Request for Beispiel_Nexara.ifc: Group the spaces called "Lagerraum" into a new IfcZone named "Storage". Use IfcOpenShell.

First a look at what the model holds.

```python
import ifcopenshell

model = ifcopenshell.open("Beispiel_Nexara.ifc")
print(model.schema)
seen = {}
for space in model.by_type("IfcSpace"):
    seen[space.LongName] = seen.get(space.LongName, 0) + 1
for name, count in sorted(seen.items(), key=str):
    print(count, "x", name)
print("zones:", [z.Name for z in model.by_type("IfcZone")][:20])
```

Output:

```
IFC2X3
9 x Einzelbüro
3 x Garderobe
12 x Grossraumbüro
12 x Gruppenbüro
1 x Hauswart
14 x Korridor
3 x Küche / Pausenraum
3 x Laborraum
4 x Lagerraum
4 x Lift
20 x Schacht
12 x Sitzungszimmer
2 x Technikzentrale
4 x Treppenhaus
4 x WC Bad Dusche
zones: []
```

```python
import ifcopenshell
import ifcopenshell.api.group
import ifcopenshell.api.root

model = ifcopenshell.open("Beispiel_Nexara.ifc")

names = {"Lagerraum"}
spaces = [s for s in model.by_type("IfcSpace") if s.LongName in names]

zone = ifcopenshell.api.root.create_entity(model, ifc_class="IfcZone", name="Storage")
ifcopenshell.api.group.assign_group(model, products=spaces, group=zone)
print(len(spaces), "spaces in", zone.Name)

model.write("Beispiel_Nexara_rev.ifc")
```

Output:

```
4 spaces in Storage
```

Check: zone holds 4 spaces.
